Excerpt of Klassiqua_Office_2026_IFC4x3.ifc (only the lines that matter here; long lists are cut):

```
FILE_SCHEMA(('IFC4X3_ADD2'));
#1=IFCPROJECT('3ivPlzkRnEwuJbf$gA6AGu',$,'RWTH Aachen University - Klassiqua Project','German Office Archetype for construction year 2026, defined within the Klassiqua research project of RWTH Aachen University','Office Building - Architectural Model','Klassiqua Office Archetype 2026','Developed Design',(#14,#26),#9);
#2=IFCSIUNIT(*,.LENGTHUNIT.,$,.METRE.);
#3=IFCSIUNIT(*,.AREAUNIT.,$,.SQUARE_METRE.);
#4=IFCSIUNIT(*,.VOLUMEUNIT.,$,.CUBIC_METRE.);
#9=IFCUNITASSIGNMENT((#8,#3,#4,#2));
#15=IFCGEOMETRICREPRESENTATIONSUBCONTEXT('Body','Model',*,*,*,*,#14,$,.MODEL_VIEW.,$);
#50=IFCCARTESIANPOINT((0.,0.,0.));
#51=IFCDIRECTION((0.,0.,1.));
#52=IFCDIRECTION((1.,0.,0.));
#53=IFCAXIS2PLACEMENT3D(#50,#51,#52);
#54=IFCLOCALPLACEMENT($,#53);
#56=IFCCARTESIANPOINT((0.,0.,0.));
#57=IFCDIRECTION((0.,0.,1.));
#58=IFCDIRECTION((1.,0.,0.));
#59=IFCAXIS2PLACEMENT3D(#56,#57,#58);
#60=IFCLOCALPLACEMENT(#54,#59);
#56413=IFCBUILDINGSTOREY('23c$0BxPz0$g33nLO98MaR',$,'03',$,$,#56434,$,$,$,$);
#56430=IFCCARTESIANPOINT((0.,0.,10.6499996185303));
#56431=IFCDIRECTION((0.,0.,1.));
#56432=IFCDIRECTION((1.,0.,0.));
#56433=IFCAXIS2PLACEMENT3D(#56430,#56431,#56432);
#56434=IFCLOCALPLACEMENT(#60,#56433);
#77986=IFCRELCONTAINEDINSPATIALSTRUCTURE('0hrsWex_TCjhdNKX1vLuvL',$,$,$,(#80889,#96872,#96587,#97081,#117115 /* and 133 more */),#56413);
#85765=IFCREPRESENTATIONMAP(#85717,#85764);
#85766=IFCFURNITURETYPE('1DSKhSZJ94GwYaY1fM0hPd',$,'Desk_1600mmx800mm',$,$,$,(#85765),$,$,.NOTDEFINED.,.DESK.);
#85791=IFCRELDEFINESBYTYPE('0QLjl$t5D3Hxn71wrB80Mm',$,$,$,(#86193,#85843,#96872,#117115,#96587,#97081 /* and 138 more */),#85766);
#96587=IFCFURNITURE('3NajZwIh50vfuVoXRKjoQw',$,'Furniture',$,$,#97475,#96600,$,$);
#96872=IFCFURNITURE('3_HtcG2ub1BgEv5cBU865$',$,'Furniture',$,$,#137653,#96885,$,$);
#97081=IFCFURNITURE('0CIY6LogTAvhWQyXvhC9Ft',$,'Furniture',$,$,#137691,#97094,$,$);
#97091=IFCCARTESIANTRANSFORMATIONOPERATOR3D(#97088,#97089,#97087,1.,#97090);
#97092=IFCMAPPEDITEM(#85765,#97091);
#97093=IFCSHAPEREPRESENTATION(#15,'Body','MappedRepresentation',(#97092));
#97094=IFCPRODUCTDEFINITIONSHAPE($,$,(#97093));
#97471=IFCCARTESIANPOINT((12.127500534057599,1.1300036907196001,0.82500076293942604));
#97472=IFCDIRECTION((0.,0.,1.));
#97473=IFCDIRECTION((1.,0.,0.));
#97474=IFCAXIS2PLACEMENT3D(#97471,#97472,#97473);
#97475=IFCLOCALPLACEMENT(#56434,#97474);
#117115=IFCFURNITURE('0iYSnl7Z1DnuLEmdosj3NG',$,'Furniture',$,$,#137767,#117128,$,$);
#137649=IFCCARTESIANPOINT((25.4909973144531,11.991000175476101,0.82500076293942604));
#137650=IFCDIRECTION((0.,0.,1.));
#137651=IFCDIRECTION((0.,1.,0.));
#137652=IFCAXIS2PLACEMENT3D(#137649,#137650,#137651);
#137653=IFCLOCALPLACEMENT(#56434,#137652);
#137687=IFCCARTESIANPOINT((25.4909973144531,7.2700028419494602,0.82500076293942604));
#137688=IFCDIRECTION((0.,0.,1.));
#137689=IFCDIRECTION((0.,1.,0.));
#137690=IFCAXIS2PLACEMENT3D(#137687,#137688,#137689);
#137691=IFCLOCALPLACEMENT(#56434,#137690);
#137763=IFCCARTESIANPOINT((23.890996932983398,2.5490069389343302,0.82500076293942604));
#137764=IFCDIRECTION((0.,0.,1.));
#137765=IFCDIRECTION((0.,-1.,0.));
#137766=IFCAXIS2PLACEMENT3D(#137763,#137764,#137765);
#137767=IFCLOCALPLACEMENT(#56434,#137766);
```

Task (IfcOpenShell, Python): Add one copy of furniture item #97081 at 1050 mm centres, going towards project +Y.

```python
import numpy as np
import ifcopenshell
import ifcopenshell.api.geometry
import ifcopenshell.api.root
import ifcopenshell.util.element
import ifcopenshell.util.placement

model = ifcopenshell.open("Klassiqua_Office_2026_IFC4x3.ifc")

source = model.by_guid("0CIY6LogTAvhWQyXvhC9Ft")
base = ifcopenshell.util.placement.get_local_placement(source.ObjectPlacement)
step = np.array([0.0, 1.0, 0.0]) * 1.05

for i in range(1, 2):
    copy = ifcopenshell.api.root.copy_class(model, product=source)
    copy.Representation = ifcopenshell.util.element.copy_deep(
        model, source.Representation, exclude=["IfcGeometricRepresentationContext", "IfcRepresentationMap"]
    )
    matrix = base.copy()
    matrix[:3, 3] += i * step
    print("added at", matrix[:3, 3].round(3) + 0.0)
    ifcopenshell.api.geometry.edit_object_placement(model, product=copy, matrix=matrix, is_si=False)

model.write("Klassiqua_Office_2026_IFC4x3_edited.ifc")
```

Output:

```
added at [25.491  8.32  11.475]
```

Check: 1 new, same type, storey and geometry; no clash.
